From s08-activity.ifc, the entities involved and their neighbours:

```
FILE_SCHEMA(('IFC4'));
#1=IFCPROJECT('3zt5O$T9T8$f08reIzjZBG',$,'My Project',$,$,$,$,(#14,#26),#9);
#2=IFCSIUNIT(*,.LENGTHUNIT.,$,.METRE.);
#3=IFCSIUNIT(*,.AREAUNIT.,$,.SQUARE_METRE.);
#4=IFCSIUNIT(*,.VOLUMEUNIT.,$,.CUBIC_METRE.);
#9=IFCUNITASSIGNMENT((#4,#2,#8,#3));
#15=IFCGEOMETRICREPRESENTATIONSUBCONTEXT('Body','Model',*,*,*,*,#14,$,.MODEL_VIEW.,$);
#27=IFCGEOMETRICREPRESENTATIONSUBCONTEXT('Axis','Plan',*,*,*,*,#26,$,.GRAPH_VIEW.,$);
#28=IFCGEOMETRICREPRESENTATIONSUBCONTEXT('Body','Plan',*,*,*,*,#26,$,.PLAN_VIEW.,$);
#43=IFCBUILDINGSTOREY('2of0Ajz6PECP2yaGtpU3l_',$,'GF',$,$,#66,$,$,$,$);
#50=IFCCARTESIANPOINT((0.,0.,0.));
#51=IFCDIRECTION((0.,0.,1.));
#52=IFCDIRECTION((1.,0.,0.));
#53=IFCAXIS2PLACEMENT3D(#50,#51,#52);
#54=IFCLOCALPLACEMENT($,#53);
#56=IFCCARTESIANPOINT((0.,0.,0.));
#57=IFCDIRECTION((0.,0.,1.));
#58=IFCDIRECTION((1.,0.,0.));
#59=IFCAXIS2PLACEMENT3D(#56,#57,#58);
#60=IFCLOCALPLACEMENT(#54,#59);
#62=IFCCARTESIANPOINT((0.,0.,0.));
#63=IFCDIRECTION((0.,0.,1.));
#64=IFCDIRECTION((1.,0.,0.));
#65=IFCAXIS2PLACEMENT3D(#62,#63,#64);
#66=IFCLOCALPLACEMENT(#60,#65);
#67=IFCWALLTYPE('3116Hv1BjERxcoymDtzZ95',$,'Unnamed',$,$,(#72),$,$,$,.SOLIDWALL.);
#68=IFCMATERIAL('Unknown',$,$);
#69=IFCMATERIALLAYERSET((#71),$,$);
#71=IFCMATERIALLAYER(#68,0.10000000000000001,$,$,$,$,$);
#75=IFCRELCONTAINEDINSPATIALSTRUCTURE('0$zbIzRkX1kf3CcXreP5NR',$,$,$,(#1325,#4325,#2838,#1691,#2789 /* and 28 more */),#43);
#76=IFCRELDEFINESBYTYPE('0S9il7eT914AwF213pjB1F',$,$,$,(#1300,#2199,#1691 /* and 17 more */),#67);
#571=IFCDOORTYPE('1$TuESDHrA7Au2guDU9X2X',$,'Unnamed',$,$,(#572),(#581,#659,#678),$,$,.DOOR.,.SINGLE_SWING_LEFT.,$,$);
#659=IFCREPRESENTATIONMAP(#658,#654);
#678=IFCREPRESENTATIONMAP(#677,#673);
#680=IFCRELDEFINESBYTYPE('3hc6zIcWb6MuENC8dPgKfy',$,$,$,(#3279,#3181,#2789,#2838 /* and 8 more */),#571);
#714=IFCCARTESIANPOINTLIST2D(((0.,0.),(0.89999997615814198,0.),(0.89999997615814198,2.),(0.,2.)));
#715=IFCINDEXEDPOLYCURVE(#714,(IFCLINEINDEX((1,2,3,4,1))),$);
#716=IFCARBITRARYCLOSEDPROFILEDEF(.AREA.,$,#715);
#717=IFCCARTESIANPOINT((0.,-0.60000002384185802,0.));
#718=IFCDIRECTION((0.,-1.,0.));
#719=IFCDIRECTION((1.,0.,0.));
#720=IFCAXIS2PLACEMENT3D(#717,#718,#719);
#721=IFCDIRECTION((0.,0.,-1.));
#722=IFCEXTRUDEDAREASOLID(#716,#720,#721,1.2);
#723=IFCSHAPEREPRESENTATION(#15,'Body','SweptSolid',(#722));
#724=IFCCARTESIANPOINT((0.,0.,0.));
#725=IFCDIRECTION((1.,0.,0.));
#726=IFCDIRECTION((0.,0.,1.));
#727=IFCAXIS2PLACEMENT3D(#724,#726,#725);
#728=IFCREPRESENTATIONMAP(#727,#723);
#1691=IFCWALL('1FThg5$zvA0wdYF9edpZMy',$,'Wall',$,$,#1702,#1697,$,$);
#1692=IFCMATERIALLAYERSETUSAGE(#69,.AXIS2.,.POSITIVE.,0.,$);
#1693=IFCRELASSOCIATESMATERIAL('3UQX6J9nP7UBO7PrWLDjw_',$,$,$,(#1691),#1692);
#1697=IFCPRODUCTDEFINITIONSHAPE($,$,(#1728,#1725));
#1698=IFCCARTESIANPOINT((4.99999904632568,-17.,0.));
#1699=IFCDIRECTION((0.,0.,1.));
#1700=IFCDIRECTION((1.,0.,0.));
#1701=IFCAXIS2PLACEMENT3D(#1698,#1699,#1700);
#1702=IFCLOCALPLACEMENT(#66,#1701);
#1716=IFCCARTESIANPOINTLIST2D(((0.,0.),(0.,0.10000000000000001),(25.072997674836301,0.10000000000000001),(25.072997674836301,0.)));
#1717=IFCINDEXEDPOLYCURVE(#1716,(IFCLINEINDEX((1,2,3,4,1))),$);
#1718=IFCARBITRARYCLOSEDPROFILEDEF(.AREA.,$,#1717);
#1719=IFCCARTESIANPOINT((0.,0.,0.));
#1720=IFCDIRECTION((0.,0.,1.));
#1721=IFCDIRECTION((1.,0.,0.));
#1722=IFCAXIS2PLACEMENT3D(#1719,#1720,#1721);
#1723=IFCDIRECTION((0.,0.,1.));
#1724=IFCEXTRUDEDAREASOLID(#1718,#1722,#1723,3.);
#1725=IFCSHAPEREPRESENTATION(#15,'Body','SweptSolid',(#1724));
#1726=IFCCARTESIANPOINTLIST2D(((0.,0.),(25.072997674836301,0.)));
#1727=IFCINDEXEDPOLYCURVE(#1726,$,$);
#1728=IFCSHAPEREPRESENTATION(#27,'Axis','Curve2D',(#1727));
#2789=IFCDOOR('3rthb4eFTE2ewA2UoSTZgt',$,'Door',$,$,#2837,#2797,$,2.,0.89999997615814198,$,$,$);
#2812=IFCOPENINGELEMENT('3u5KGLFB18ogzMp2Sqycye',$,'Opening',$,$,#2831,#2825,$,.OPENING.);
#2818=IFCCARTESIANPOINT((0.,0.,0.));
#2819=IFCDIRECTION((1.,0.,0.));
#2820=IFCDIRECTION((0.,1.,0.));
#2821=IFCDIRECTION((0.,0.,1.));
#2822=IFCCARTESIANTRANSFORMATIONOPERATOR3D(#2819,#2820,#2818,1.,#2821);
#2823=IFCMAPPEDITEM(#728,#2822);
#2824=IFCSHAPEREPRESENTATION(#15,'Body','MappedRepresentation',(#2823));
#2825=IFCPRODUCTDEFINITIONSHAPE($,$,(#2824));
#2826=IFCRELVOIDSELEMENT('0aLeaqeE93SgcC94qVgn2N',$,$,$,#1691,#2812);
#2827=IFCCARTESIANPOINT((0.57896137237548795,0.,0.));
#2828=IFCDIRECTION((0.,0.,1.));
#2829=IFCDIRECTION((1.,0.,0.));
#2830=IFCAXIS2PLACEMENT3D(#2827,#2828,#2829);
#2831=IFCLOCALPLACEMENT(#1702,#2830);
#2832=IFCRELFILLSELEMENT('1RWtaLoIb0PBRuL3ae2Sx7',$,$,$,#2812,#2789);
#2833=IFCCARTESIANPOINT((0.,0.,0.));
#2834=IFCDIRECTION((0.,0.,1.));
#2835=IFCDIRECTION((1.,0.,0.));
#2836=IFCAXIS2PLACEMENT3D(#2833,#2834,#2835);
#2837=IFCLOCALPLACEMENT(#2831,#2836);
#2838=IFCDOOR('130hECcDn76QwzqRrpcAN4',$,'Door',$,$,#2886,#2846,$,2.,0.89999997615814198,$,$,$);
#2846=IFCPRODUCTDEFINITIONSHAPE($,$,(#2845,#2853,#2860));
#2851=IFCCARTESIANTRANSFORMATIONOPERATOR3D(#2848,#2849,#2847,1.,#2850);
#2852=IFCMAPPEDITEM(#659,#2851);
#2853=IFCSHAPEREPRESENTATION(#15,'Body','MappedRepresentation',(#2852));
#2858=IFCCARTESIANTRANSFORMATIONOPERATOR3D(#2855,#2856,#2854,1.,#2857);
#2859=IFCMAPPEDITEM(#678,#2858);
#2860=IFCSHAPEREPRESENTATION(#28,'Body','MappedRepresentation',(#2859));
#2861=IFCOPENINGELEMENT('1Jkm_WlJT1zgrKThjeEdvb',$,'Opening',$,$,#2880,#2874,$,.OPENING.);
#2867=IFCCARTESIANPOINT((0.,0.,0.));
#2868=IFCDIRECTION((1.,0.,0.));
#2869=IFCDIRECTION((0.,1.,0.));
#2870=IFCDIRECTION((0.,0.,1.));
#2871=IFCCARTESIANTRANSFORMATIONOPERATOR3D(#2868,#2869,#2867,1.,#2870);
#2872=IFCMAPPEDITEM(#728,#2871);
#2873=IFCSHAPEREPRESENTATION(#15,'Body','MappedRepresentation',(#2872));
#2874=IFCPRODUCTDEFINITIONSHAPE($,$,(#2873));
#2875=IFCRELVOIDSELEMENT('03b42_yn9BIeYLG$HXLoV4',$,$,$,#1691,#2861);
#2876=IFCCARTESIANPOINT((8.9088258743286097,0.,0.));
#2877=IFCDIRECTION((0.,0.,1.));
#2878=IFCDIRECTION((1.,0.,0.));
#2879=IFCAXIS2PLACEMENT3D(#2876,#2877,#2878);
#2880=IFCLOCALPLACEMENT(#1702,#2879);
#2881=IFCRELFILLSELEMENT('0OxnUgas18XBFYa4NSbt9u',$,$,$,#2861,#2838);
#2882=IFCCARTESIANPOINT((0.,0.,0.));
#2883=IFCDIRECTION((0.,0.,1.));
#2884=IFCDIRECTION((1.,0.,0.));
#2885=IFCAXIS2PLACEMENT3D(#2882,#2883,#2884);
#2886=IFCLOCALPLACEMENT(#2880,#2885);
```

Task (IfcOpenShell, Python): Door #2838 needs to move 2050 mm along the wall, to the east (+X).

```python
import ifcopenshell
import ifcopenshell.api.geometry
import ifcopenshell.util.placement
import ifcopenshell.util.unit

model = ifcopenshell.open("s08-activity.ifc")
unit_scale = ifcopenshell.util.unit.calculate_unit_scale(model)

door = model.by_guid("130hECcDn76QwzqRrpcAN4")
opening = door.FillsVoids[0].RelatingOpeningElement
wall = opening.VoidsElements[0].RelatingBuildingElement

wall_matrix = ifcopenshell.util.placement.get_local_placement(wall.ObjectPlacement)
shift = wall_matrix[:3, 0] * 2.05 / unit_scale
before = ifcopenshell.util.placement.get_local_placement(door.ObjectPlacement)[:3, 3].copy()

# The door is placed relative to its opening, so it follows when the opening moves.
matrix = ifcopenshell.util.placement.get_local_placement(opening.ObjectPlacement)
matrix[:3, 3] += shift
ifcopenshell.api.geometry.edit_object_placement(
    model, product=opening, matrix=matrix, is_si=False, should_transform_children=True
)

after = ifcopenshell.util.placement.get_local_placement(door.ObjectPlacement)[:3, 3]
print("door moved by", (after - before).round(3) + 0.0)

model.write("s08-activity_edited.ifc")
```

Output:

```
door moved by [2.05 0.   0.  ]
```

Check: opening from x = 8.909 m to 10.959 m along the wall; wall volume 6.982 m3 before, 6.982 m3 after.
